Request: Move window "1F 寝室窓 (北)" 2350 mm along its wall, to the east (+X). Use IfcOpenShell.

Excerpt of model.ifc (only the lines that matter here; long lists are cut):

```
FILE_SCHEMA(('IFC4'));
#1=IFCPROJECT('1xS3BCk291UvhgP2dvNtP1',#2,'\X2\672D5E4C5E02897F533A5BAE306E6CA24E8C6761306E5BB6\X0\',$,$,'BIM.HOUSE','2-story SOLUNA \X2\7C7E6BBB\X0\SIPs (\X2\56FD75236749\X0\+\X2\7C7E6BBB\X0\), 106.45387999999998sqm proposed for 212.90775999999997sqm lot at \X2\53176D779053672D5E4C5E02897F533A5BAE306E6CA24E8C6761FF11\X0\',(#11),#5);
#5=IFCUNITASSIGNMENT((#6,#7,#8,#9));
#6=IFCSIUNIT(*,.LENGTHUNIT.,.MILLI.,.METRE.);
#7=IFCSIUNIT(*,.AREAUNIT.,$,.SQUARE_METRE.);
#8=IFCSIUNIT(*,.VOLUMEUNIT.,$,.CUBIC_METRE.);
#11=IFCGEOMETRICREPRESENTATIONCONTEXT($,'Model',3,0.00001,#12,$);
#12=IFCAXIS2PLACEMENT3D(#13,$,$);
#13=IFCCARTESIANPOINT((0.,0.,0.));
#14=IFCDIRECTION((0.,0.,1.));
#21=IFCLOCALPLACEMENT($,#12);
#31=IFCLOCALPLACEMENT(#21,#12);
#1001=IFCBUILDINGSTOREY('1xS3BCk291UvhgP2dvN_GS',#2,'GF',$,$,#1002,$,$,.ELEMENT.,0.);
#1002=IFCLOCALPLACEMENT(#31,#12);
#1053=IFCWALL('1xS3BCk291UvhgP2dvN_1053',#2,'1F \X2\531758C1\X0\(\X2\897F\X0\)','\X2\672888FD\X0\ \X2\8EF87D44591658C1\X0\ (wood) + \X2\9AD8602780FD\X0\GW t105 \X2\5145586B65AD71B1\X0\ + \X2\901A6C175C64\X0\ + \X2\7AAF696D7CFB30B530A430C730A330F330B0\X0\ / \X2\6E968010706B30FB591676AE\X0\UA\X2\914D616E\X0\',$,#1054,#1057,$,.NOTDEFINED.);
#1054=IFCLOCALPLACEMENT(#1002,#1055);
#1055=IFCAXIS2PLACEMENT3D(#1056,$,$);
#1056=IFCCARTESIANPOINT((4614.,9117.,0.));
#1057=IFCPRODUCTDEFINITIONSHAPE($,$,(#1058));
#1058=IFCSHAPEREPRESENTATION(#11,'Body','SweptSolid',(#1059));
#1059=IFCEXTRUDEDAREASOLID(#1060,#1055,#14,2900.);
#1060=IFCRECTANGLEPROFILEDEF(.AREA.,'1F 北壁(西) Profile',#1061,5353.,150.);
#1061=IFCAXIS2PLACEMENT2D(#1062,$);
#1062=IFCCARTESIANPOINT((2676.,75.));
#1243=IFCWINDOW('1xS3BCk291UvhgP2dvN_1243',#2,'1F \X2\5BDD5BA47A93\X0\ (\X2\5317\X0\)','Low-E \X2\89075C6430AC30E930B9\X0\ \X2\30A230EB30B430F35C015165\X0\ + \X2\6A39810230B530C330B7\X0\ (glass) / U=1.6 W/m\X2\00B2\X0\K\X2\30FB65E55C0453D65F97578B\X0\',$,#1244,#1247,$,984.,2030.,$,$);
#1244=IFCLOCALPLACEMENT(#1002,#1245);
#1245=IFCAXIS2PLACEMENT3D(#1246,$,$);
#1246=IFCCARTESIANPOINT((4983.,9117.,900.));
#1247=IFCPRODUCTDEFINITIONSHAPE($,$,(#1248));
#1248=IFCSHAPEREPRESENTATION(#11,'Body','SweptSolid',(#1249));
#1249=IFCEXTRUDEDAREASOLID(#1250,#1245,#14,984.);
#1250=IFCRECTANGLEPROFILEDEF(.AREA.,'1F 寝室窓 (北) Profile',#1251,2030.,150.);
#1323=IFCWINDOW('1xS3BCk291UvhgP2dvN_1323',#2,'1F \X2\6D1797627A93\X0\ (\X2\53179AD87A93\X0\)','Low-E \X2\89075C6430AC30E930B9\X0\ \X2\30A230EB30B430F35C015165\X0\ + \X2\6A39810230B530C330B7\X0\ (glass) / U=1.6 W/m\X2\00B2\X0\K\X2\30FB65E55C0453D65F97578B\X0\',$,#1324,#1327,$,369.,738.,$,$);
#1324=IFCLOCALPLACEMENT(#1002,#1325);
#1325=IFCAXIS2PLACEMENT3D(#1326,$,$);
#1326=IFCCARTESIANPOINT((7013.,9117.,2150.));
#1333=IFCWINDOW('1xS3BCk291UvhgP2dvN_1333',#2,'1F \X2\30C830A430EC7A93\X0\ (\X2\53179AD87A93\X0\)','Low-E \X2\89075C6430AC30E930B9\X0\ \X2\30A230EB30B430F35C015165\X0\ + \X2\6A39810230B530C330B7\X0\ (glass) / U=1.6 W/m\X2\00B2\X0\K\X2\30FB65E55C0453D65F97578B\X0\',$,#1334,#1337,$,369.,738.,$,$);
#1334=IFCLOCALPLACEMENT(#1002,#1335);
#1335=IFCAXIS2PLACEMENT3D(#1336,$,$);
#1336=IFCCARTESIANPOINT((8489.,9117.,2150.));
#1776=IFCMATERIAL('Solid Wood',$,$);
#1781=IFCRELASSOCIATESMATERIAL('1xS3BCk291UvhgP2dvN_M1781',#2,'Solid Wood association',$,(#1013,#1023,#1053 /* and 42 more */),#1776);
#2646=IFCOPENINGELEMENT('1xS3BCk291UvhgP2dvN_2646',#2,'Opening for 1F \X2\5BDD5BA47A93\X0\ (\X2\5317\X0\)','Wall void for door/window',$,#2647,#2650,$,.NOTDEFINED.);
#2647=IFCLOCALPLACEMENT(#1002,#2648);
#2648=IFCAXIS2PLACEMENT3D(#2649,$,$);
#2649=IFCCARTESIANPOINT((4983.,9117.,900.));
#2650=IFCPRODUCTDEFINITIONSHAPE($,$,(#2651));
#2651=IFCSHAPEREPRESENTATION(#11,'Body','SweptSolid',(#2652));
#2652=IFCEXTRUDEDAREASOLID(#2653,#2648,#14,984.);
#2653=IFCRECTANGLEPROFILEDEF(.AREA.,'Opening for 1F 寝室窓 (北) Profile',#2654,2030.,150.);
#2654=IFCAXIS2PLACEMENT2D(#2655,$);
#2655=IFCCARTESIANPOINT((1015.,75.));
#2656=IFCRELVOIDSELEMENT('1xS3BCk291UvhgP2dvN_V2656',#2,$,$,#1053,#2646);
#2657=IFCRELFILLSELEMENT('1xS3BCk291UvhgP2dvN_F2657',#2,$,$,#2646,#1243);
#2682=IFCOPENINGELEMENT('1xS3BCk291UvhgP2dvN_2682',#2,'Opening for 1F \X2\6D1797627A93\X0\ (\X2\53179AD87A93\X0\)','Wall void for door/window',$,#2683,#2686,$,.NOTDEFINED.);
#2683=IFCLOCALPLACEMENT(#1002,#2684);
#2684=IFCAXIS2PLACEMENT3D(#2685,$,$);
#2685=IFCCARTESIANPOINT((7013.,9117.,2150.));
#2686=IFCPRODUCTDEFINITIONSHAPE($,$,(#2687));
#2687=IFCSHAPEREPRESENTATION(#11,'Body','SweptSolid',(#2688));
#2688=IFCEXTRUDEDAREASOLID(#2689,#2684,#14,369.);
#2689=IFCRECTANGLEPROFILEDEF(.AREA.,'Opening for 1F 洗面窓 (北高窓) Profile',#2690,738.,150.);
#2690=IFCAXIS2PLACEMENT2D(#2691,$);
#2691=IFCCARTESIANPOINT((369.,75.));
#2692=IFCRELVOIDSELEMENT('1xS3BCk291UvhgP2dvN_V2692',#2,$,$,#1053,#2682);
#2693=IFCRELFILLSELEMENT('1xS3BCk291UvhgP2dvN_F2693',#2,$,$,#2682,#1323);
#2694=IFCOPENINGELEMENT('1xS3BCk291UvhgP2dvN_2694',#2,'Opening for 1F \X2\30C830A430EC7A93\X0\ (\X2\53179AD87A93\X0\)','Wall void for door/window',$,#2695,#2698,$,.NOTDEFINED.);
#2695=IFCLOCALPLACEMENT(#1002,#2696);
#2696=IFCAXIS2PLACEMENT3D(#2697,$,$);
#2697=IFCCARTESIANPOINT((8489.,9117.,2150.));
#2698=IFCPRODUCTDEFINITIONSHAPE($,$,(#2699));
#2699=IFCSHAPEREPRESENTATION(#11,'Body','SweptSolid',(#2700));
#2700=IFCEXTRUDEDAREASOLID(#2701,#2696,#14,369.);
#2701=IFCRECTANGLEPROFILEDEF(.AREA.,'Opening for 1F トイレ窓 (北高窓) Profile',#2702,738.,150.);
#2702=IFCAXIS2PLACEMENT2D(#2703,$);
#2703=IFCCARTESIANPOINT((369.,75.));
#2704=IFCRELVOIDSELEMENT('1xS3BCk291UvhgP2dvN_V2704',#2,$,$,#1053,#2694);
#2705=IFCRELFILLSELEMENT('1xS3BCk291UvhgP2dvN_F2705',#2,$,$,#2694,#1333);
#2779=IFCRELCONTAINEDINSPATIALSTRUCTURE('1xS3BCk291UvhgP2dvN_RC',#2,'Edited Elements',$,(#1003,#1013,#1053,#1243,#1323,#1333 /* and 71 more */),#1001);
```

```python
import ifcopenshell
import ifcopenshell.api.geometry
import ifcopenshell.util.placement
import ifcopenshell.util.unit

model = ifcopenshell.open("model.ifc")
unit_scale = ifcopenshell.util.unit.calculate_unit_scale(model)

window = model.by_guid("1xS3BCk291UvhgP2dvN_1243")
opening = window.FillsVoids[0].RelatingOpeningElement
wall = opening.VoidsElements[0].RelatingBuildingElement

wall_matrix = ifcopenshell.util.placement.get_local_placement(wall.ObjectPlacement)
shift = wall_matrix[:3, 0] * 2.35 / unit_scale
before = ifcopenshell.util.placement.get_local_placement(window.ObjectPlacement)[:3, 3].copy()

# The window is not placed relative to its opening, so move both.
for product in (opening, window):
    matrix = ifcopenshell.util.placement.get_local_placement(product.ObjectPlacement)
    matrix[:3, 3] += shift
    ifcopenshell.api.geometry.edit_object_placement(model, product=product, matrix=matrix, is_si=False)

after = ifcopenshell.util.placement.get_local_placement(window.ObjectPlacement)[:3, 3]
print("window moved by", (after - before).round(3) + 0.0)

model.write("model_edited.ifc")
```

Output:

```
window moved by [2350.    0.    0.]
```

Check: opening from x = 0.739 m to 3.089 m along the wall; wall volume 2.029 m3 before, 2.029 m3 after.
